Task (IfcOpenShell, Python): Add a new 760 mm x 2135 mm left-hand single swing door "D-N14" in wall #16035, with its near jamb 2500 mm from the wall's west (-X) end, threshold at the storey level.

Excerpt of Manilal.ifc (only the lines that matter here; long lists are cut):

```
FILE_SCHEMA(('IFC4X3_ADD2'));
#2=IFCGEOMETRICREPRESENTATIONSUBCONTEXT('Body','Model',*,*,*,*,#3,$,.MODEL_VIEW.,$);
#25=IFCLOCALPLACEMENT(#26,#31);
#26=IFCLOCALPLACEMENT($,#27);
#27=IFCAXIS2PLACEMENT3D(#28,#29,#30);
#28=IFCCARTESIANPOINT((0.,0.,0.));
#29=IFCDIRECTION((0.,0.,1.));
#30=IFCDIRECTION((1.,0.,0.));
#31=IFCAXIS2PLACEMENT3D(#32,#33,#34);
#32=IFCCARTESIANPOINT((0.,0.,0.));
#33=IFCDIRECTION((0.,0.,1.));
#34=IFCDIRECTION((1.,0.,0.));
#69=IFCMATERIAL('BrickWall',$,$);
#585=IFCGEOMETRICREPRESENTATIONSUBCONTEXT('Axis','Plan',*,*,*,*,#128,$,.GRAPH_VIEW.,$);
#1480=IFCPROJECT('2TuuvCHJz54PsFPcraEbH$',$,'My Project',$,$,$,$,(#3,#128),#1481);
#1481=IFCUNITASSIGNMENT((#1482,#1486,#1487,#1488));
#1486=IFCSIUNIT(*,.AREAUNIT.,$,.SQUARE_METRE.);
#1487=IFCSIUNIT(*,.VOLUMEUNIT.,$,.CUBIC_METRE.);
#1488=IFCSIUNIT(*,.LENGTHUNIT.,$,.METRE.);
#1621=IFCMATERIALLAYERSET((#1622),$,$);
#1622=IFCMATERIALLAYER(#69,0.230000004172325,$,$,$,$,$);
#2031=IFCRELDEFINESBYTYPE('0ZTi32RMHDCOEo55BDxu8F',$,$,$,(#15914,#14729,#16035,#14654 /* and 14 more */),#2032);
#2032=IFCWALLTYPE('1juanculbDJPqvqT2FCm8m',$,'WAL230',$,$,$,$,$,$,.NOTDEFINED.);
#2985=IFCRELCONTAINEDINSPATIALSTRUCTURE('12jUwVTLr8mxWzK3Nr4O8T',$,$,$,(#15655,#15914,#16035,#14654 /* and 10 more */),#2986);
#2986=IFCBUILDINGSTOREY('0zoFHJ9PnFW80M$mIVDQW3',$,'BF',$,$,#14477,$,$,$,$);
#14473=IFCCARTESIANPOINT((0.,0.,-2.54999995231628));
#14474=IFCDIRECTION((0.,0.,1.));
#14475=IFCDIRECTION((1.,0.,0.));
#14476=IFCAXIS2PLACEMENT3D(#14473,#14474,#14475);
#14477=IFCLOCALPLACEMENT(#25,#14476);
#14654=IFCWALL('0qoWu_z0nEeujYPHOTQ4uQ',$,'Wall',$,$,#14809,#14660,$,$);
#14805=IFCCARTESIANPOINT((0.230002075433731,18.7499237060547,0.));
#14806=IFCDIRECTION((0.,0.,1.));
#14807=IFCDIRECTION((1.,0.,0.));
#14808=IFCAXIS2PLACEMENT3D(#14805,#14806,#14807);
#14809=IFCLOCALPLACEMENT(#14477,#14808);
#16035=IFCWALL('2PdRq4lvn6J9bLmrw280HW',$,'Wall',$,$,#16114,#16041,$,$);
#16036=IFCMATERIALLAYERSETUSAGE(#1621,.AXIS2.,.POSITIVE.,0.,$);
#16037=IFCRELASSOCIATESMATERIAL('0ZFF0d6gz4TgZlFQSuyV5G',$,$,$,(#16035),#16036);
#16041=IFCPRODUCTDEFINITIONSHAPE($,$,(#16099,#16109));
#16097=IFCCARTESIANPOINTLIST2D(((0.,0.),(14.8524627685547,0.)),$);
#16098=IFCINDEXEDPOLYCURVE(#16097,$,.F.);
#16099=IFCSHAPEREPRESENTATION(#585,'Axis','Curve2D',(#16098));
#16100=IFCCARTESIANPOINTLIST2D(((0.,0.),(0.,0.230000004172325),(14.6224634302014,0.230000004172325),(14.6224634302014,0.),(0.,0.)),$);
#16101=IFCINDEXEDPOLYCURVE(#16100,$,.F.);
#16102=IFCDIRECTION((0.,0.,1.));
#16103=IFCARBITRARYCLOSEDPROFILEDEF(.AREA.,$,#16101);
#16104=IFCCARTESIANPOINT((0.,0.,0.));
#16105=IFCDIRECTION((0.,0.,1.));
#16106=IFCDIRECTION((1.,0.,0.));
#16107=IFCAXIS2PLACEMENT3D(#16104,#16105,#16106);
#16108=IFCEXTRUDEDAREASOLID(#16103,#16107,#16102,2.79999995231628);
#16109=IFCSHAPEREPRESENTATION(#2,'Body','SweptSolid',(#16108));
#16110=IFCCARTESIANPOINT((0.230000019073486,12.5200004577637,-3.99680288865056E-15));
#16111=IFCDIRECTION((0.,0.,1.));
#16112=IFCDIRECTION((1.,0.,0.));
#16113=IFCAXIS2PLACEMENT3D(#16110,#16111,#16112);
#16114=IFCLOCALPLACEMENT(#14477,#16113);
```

```python
import numpy as np
import ifcopenshell
import ifcopenshell.api.feature
import ifcopenshell.api.geometry
import ifcopenshell.api.root
import ifcopenshell.api.spatial
import ifcopenshell.geom
import ifcopenshell.util.element
import ifcopenshell.util.placement
import ifcopenshell.util.representation
import ifcopenshell.util.shape
import ifcopenshell.util.unit

model = ifcopenshell.open("Manilal.ifc")
unit_scale = ifcopenshell.util.unit.calculate_unit_scale(model)
settings = ifcopenshell.geom.settings()


def volume(element):
    """Net volume in cubic metres, openings subtracted."""
    shape = ifcopenshell.geom.create_shape(settings, element)
    return ifcopenshell.util.shape.get_volume(shape.geometry)


wall = model.by_id(16035)
storey = ifcopenshell.util.element.get_container(wall, ifc_class="IfcBuildingStorey")
context = ifcopenshell.util.representation.get_context(model, "Model", "Body", "MODEL_VIEW")
before = volume(wall)

width, height, from_end, sill = 0.76, 2.135, 2.5, 0.0  # metres

# The wall runs along its own X axis, and the end named is its -X end.
wall_shape = ifcopenshell.geom.create_shape(settings, wall)
x, y, z = ifcopenshell.util.shape.get_vertices(wall_shape.geometry).T
start = x.min() + from_end
face, thickness = float(y.min()), float(y.max() - y.min())
wall_matrix = ifcopenshell.util.placement.get_local_placement(wall.ObjectPlacement)
level = ifcopenshell.util.placement.get_local_placement(storey.ObjectPlacement)[2, 3]


def in_wall(x, y):
    """Placement at x, y metres in the wall's axes, at sill height."""
    matrix = wall_matrix.copy()
    matrix[:, 3] = wall_matrix @ np.array([x / unit_scale, y / unit_scale, 0.0, 1.0])
    matrix[2, 3] = level + sill / unit_scale
    return matrix


# Opening: a box that overshoots both wall faces by 50 mm.
opening = ifcopenshell.api.root.create_entity(model, ifc_class="IfcOpeningElement", predefined_type="OPENING")
box = ifcopenshell.api.geometry.add_wall_representation(
    model, context=context, length=width, height=height, thickness=thickness + 0.1
)
ifcopenshell.api.geometry.assign_representation(model, product=opening, representation=box)
ifcopenshell.api.geometry.edit_object_placement(model, product=opening, matrix=in_wall(start, face - 0.05), is_si=False)
ifcopenshell.api.feature.add_feature(model, feature=opening, element=wall)

door = ifcopenshell.api.root.create_entity(model, ifc_class="IfcDoor", name="D-N14", predefined_type="DOOR")
door.OverallWidth, door.OverallHeight = width / unit_scale, height / unit_scale
door.OperationType = "SINGLE_SWING_LEFT"
body = ifcopenshell.api.geometry.add_door_representation(
    model,
    context=context,
    overall_width=door.OverallWidth,
    overall_height=door.OverallHeight,
    operation_type="SINGLE_SWING_LEFT",
    lining_properties={"LiningDepth": thickness / unit_scale, "ThresholdDepth": thickness / unit_scale},
)
ifcopenshell.api.geometry.assign_representation(model, product=door, representation=body)
ifcopenshell.api.spatial.assign_container(model, products=[door], relating_structure=storey)
ifcopenshell.api.feature.add_filling(model, opening=opening, element=door)

# The lining spans the wall, so the door starts at the wall face.
ifcopenshell.api.geometry.edit_object_placement(model, product=door, matrix=in_wall(start, face), is_si=False)

after = volume(wall)

print(f"wall volume {before:.3f} -> {after:.3f} m3")

model.write("Manilal-out.ifc")
```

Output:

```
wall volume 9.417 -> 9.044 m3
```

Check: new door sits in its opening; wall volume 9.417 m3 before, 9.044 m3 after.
